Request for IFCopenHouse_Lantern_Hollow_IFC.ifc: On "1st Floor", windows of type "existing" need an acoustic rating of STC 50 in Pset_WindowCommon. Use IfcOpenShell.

First a look at what the model holds.

```python
import ifcopenshell
import ifcopenshell.util.element

model = ifcopenshell.open("IFCopenHouse_Lantern_Hollow_IFC.ifc")
print(model.schema)
storey = next(s for s in model.by_type("IfcBuildingStorey") if s.Name == "1st Floor")
windows = [e for e in ifcopenshell.util.element.get_decomposition(storey) if e.is_a("IfcWindow")]
seen = {}
for e in windows:
    element_type = ifcopenshell.util.element.get_type(e)
    key = (element_type.Name if element_type != e and element_type else None, ifcopenshell.util.element.get_pset(e, "Pset_WindowCommon", "AcousticRating"))
    seen[key] = seen.get(key, 0) + 1
for (name, value), count in sorted(seen.items(), key=str):
    print(count, "x", name, "|", value)
```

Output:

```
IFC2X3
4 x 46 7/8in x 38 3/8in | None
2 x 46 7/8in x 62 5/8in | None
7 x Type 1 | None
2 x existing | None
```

```python
import ifcopenshell
import ifcopenshell.api.pset
import ifcopenshell.util.element

model = ifcopenshell.open("IFCopenHouse_Lantern_Hollow_IFC.ifc")

storey = next(s for s in model.by_type("IfcBuildingStorey") if s.Name == "1st Floor")
windows = [e for e in ifcopenshell.util.element.get_decomposition(storey) if e.is_a("IfcWindow")]

count = 0
for e in windows:
    element_type = ifcopenshell.util.element.get_type(e)
    if element_type in (None, e) or element_type.Name != "existing":
        continue
    # add_pset returns the element's existing set when there is one.
    pset = ifcopenshell.api.pset.add_pset(model, product=e, name="Pset_WindowCommon")
    ifcopenshell.api.pset.edit_pset(model, pset=pset, properties={"AcousticRating": "STC 50"})
    count += 1

print(count, "windows updated")

model.write("IFCopenHouse_Lantern_Hollow_IFC_rev.ifc")
```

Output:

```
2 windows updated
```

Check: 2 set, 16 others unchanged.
